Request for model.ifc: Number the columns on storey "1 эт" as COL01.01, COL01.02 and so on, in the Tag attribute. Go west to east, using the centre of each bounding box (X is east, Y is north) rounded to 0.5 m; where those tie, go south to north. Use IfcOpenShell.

First a look at what the model holds.

```python
import ifcopenshell
import ifcopenshell.util.element
import ifcopenshell.util.placement

model = ifcopenshell.open("model.ifc")
print(model.schema)
storey = next(s for s in model.by_type("IfcBuildingStorey") if s.Name == "1 эт")
columns = [e for e in ifcopenshell.util.element.get_decomposition(storey) if e.is_a("IfcColumn")]
for e in sorted(columns, key=lambda e: e.id()):
    origin = ifcopenshell.util.placement.get_local_placement(e.ObjectPlacement)[:3, 3]
    print(e.id(), e.Tag, e.Name, origin.round(2) + 0.0, sep=" | ")
```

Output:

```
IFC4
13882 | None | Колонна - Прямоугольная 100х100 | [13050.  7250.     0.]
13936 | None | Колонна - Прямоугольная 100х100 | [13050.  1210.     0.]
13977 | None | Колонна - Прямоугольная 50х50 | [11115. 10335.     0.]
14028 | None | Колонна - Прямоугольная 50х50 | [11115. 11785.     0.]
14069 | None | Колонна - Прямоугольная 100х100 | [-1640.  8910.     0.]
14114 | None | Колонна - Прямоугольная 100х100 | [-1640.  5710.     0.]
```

```python
import ifcopenshell
import ifcopenshell.geom
import ifcopenshell.util.element
import ifcopenshell.util.shape

model = ifcopenshell.open("model.ifc")
settings = ifcopenshell.geom.settings()
settings.set("use-world-coords", True)


def centre(element):
    shape = ifcopenshell.geom.create_shape(settings, element)
    return ifcopenshell.util.shape.get_bbox_centroid(shape.geometry)


storey = next(s for s in model.by_type("IfcBuildingStorey") if s.Name == "1 эт")
columns = [e for e in ifcopenshell.util.element.get_decomposition(storey) if e.is_a("IfcColumn")]

# Insertion points can sit at a corner or the storey origin, so sort by the geometry (in metres).
centres = {e: centre(e) for e in columns}
columns.sort(key=lambda e: (round(centres[e][0] / 0.5), centres[e][1]))

for i, e in enumerate(columns, start=1):
    number = f"COL01.{i:02d}"
    e.Tag = number
    print(e.id(), number)

model.write("model_updated.ifc")
```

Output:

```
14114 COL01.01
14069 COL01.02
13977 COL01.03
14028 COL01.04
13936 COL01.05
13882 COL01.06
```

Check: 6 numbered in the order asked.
